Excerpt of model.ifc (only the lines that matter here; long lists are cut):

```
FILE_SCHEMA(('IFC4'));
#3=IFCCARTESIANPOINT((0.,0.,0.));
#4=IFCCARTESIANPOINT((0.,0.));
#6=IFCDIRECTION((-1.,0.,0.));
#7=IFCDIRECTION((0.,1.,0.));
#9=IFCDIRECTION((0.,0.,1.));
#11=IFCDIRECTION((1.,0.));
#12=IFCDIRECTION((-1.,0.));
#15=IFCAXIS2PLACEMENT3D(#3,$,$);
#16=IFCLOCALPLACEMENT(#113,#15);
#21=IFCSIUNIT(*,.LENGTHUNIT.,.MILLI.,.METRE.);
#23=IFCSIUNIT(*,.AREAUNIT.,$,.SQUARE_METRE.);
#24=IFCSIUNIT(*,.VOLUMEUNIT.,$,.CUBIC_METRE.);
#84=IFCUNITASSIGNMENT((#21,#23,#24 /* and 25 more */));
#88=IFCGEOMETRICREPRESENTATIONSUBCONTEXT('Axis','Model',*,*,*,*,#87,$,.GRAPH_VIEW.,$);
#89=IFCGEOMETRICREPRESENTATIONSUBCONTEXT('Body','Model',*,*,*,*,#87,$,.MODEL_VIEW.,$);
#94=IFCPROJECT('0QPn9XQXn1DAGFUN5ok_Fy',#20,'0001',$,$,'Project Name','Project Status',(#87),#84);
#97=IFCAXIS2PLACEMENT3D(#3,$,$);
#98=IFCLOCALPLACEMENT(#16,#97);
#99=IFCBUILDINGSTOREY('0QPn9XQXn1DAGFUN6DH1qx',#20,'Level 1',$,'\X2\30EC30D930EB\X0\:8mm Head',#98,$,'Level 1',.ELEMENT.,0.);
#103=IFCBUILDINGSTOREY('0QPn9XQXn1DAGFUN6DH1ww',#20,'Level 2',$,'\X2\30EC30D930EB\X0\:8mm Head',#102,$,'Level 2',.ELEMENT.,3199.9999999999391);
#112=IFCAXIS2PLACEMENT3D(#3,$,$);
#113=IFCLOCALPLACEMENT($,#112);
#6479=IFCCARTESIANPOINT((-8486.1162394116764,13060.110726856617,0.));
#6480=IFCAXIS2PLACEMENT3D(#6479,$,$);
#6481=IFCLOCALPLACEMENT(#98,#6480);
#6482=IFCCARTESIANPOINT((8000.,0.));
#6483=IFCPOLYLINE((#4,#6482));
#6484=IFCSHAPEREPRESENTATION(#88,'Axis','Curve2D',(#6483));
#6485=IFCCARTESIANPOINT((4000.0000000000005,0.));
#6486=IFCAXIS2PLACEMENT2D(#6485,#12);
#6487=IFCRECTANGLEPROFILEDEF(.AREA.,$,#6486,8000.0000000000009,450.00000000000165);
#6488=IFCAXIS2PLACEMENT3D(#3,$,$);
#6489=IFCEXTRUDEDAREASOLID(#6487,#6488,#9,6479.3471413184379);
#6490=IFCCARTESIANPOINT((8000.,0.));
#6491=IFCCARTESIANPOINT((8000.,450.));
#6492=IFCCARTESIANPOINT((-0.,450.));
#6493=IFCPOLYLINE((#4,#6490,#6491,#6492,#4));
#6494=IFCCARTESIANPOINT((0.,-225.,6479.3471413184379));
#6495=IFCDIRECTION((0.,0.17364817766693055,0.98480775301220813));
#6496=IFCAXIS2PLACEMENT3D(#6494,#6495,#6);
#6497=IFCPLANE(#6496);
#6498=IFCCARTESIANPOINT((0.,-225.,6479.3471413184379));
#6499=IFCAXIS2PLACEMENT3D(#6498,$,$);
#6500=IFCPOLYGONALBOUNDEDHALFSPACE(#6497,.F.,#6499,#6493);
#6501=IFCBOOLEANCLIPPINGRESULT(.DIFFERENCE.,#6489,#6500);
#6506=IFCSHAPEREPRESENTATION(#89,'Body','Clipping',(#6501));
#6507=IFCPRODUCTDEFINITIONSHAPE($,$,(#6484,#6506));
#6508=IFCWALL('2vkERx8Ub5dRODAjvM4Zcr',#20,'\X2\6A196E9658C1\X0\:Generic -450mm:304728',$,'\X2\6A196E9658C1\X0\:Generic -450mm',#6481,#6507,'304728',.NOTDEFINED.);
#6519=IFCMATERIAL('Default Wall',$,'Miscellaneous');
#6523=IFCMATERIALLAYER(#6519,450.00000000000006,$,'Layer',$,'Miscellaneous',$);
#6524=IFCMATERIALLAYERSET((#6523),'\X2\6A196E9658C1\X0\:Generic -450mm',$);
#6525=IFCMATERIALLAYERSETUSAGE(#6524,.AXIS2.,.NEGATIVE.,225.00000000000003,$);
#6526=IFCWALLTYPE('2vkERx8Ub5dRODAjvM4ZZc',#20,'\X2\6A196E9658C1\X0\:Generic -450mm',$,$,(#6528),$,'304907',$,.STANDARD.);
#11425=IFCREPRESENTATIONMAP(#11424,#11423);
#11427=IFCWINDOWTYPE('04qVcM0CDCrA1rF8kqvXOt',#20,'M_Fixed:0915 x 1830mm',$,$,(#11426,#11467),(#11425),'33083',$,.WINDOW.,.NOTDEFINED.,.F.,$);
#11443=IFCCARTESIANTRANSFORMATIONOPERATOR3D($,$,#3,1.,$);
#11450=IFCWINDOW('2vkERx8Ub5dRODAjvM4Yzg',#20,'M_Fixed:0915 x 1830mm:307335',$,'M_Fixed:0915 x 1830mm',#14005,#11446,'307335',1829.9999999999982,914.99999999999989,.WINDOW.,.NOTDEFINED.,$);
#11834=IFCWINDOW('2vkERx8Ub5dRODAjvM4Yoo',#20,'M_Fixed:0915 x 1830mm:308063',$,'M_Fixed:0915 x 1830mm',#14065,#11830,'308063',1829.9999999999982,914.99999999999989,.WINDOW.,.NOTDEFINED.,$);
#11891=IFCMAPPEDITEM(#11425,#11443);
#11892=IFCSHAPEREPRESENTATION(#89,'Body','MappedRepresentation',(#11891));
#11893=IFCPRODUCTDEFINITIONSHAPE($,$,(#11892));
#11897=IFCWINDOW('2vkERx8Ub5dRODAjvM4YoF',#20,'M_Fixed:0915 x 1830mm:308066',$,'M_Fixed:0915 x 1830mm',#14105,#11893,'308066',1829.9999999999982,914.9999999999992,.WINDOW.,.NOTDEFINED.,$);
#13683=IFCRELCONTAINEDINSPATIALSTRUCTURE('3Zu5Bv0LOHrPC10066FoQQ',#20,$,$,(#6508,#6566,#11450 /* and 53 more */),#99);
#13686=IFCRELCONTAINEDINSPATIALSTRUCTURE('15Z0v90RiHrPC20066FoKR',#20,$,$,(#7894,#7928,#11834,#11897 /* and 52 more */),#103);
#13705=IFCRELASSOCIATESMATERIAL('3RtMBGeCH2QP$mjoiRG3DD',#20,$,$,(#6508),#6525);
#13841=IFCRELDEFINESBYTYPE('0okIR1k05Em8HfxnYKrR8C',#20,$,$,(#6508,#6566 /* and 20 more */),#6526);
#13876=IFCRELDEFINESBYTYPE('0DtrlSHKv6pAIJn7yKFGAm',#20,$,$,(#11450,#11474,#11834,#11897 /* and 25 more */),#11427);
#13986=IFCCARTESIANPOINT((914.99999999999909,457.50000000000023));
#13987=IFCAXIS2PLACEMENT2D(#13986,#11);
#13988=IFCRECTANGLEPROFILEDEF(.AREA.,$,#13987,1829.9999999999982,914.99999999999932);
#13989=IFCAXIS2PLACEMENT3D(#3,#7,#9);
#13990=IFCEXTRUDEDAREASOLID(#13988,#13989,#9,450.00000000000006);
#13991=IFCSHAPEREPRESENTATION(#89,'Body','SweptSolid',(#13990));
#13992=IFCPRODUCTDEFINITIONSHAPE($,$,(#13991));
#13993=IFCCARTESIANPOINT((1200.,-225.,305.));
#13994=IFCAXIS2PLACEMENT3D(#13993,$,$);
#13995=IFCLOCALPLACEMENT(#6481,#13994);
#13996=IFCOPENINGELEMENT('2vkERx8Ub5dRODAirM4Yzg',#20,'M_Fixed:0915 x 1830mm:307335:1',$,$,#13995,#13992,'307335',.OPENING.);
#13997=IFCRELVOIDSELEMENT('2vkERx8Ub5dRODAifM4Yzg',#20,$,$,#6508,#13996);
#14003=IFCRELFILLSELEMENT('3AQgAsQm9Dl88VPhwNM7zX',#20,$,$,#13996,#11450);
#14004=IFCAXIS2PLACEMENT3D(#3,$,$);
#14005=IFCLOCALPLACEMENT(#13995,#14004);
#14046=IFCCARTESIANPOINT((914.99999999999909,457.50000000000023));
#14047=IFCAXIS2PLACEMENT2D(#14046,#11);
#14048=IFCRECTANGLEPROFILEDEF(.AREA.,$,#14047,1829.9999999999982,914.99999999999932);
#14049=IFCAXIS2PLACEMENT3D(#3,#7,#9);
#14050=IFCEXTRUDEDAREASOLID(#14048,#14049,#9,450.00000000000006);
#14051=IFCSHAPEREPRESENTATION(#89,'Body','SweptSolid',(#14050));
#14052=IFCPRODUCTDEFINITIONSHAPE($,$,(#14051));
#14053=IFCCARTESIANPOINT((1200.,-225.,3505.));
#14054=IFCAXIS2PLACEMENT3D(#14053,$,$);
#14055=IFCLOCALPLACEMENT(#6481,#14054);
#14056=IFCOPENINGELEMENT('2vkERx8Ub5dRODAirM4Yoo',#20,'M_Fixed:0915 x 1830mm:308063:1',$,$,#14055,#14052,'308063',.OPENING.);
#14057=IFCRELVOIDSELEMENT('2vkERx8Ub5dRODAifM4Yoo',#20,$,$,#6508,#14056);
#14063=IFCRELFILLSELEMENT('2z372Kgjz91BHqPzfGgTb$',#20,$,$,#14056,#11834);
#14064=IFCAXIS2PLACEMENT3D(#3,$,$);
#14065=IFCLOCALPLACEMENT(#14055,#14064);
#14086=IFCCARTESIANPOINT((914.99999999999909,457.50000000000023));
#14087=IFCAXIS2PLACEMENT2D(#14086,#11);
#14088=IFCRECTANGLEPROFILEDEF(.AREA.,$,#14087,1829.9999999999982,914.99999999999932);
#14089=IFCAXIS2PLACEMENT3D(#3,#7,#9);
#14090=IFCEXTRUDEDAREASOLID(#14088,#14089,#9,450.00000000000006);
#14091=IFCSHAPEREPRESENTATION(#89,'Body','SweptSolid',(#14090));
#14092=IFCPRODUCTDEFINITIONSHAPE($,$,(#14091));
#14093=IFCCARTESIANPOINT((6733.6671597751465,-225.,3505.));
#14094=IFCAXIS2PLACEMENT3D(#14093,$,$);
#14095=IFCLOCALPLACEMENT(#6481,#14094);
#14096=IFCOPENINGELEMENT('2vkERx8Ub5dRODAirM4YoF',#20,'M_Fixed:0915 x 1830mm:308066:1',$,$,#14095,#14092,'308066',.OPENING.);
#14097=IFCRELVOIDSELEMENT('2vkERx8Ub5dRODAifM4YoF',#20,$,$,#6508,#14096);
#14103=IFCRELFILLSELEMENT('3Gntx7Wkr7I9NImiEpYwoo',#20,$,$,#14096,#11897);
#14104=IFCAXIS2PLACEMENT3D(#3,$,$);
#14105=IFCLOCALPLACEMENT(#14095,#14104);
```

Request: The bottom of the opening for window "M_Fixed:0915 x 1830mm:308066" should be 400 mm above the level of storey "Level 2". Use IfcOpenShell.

```python
import numpy as np
import ifcopenshell
import ifcopenshell.api.geometry
import ifcopenshell.geom
import ifcopenshell.util.element
import ifcopenshell.util.placement
import ifcopenshell.util.shape
import ifcopenshell.util.unit

model = ifcopenshell.open("model.ifc")
unit_scale = ifcopenshell.util.unit.calculate_unit_scale(model)

window = model.by_guid("2vkERx8Ub5dRODAjvM4YoF")
opening = window.FillsVoids[0].RelatingOpeningElement
storey = ifcopenshell.util.element.get_container(window, ifc_class="IfcBuildingStorey")
level = ifcopenshell.util.placement.get_local_placement(storey.ObjectPlacement)[2, 3]

# The opening's origin need not be at the sill, so measure its lowest point.
shape = ifcopenshell.geom.create_shape(ifcopenshell.geom.settings(), opening)
bottom = ifcopenshell.util.shape.get_shape_bottom_elevation(shape, shape.geometry) / unit_scale
dz = level + 0.4 / unit_scale - bottom

shift = np.array([0.0, 0.0, dz])
# The window is placed relative to its opening, so it follows when the opening moves.
matrix = ifcopenshell.util.placement.get_local_placement(opening.ObjectPlacement)
matrix[:3, 3] += shift
ifcopenshell.api.geometry.edit_object_placement(
    model, product=opening, matrix=matrix, is_si=False, should_transform_children=True
)

print(f"moved by {dz * unit_scale:+.3f} m")

model.write("model_v2.ifc")
```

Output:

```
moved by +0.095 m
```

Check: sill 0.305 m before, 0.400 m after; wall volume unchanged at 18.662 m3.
